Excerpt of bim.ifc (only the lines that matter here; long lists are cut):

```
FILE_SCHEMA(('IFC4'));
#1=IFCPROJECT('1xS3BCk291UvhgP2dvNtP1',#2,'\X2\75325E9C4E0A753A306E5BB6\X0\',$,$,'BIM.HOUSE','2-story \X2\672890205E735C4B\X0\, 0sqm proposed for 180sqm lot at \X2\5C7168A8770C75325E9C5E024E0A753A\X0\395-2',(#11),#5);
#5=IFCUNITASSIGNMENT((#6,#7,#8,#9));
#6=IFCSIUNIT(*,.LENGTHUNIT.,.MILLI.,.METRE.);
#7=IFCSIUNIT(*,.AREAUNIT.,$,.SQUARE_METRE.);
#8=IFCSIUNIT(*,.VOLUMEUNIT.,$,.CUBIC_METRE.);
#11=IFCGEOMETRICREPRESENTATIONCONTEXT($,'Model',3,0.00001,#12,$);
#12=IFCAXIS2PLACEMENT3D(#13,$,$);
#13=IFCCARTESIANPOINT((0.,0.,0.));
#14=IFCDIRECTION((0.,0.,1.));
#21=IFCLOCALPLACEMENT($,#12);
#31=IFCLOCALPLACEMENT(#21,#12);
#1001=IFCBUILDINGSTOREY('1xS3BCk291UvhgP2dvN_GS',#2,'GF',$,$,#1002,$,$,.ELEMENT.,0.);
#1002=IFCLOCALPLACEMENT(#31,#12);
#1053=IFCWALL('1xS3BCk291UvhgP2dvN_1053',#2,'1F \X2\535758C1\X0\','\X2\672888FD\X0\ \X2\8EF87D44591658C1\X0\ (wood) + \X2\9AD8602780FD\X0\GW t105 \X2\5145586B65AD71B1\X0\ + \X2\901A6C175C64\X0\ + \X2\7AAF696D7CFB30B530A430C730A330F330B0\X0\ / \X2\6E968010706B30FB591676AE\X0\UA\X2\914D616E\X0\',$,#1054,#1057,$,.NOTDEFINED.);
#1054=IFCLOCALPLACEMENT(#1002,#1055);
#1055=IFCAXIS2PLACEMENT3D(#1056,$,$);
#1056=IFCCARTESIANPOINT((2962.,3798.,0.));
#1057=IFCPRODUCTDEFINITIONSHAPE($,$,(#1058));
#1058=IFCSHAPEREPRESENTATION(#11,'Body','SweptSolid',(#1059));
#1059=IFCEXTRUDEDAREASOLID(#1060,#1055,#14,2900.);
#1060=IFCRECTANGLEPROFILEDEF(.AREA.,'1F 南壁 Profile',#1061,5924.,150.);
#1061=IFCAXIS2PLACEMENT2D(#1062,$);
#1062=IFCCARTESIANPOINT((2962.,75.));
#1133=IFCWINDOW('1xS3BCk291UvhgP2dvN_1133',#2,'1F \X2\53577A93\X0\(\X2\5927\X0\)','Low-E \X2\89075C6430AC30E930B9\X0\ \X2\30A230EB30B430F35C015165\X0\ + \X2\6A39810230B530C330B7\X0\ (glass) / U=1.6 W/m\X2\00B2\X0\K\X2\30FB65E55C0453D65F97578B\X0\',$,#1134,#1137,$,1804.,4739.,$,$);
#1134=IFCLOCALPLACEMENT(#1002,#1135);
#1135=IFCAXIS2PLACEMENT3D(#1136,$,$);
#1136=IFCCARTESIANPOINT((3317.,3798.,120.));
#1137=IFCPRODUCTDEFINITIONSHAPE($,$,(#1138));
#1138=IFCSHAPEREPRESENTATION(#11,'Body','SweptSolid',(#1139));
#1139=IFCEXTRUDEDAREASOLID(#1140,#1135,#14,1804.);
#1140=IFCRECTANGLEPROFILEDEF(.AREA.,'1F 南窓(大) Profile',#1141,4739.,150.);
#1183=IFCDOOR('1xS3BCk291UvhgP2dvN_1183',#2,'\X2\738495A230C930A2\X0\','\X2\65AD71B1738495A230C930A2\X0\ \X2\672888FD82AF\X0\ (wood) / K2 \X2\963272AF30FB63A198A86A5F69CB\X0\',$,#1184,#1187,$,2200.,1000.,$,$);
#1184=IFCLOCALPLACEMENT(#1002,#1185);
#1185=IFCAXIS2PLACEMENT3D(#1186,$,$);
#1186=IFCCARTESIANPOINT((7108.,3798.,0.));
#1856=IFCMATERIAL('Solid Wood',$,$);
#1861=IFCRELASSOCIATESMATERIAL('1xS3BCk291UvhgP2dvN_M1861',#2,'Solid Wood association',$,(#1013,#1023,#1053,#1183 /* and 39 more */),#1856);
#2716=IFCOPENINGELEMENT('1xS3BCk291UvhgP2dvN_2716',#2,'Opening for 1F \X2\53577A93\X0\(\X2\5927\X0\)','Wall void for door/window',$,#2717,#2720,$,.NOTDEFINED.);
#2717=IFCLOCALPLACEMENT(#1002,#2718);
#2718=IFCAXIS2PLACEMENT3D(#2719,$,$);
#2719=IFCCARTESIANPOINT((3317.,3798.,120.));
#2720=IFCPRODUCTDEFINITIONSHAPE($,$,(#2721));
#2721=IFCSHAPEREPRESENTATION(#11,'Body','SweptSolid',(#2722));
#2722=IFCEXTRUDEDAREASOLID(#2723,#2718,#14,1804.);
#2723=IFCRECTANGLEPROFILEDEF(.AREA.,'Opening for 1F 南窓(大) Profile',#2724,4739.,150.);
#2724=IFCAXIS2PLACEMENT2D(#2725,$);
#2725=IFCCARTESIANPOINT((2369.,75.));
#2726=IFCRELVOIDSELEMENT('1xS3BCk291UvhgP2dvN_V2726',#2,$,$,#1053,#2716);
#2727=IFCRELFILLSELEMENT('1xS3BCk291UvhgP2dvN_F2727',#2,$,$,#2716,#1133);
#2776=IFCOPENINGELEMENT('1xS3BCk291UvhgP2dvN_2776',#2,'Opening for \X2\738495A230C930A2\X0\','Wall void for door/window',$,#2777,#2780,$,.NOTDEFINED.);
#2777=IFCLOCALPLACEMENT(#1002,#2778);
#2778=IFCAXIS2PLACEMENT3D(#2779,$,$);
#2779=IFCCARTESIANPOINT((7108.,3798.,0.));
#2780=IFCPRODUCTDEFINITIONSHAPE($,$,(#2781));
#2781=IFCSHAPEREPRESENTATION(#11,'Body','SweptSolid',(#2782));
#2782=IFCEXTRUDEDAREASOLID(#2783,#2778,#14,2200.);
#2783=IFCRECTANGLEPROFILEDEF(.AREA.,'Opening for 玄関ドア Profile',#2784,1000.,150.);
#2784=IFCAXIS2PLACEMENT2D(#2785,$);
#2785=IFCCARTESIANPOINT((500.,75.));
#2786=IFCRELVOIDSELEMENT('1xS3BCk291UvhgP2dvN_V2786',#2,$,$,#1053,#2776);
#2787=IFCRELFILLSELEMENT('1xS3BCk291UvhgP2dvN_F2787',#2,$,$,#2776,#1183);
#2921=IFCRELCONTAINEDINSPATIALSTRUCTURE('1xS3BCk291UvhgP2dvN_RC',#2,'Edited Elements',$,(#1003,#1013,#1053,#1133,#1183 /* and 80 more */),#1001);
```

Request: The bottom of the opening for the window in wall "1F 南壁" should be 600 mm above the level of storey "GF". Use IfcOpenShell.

```python
import numpy as np
import ifcopenshell
import ifcopenshell.api.geometry
import ifcopenshell.geom
import ifcopenshell.util.element
import ifcopenshell.util.placement
import ifcopenshell.util.shape
import ifcopenshell.util.unit

model = ifcopenshell.open("bim.ifc")
unit_scale = ifcopenshell.util.unit.calculate_unit_scale(model)

window = model.by_guid("1xS3BCk291UvhgP2dvN_1133")
opening = window.FillsVoids[0].RelatingOpeningElement
storey = ifcopenshell.util.element.get_container(window, ifc_class="IfcBuildingStorey")
level = ifcopenshell.util.placement.get_local_placement(storey.ObjectPlacement)[2, 3]

# The opening's origin need not be at the sill, so measure its lowest point.
shape = ifcopenshell.geom.create_shape(ifcopenshell.geom.settings(), opening)
bottom = ifcopenshell.util.shape.get_shape_bottom_elevation(shape, shape.geometry) / unit_scale
dz = level + 0.6 / unit_scale - bottom

shift = np.array([0.0, 0.0, dz])
# The window is not placed relative to its opening, so move both.
for product in (opening, window):
    matrix = ifcopenshell.util.placement.get_local_placement(product.ObjectPlacement)
    matrix[:3, 3] += shift
    ifcopenshell.api.geometry.edit_object_placement(model, product=product, matrix=matrix, is_si=False)

print(f"moved by {dz * unit_scale:+.3f} m")

model.write("bim_rev.ifc")
```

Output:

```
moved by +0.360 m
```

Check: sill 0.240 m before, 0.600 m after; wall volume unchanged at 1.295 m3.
